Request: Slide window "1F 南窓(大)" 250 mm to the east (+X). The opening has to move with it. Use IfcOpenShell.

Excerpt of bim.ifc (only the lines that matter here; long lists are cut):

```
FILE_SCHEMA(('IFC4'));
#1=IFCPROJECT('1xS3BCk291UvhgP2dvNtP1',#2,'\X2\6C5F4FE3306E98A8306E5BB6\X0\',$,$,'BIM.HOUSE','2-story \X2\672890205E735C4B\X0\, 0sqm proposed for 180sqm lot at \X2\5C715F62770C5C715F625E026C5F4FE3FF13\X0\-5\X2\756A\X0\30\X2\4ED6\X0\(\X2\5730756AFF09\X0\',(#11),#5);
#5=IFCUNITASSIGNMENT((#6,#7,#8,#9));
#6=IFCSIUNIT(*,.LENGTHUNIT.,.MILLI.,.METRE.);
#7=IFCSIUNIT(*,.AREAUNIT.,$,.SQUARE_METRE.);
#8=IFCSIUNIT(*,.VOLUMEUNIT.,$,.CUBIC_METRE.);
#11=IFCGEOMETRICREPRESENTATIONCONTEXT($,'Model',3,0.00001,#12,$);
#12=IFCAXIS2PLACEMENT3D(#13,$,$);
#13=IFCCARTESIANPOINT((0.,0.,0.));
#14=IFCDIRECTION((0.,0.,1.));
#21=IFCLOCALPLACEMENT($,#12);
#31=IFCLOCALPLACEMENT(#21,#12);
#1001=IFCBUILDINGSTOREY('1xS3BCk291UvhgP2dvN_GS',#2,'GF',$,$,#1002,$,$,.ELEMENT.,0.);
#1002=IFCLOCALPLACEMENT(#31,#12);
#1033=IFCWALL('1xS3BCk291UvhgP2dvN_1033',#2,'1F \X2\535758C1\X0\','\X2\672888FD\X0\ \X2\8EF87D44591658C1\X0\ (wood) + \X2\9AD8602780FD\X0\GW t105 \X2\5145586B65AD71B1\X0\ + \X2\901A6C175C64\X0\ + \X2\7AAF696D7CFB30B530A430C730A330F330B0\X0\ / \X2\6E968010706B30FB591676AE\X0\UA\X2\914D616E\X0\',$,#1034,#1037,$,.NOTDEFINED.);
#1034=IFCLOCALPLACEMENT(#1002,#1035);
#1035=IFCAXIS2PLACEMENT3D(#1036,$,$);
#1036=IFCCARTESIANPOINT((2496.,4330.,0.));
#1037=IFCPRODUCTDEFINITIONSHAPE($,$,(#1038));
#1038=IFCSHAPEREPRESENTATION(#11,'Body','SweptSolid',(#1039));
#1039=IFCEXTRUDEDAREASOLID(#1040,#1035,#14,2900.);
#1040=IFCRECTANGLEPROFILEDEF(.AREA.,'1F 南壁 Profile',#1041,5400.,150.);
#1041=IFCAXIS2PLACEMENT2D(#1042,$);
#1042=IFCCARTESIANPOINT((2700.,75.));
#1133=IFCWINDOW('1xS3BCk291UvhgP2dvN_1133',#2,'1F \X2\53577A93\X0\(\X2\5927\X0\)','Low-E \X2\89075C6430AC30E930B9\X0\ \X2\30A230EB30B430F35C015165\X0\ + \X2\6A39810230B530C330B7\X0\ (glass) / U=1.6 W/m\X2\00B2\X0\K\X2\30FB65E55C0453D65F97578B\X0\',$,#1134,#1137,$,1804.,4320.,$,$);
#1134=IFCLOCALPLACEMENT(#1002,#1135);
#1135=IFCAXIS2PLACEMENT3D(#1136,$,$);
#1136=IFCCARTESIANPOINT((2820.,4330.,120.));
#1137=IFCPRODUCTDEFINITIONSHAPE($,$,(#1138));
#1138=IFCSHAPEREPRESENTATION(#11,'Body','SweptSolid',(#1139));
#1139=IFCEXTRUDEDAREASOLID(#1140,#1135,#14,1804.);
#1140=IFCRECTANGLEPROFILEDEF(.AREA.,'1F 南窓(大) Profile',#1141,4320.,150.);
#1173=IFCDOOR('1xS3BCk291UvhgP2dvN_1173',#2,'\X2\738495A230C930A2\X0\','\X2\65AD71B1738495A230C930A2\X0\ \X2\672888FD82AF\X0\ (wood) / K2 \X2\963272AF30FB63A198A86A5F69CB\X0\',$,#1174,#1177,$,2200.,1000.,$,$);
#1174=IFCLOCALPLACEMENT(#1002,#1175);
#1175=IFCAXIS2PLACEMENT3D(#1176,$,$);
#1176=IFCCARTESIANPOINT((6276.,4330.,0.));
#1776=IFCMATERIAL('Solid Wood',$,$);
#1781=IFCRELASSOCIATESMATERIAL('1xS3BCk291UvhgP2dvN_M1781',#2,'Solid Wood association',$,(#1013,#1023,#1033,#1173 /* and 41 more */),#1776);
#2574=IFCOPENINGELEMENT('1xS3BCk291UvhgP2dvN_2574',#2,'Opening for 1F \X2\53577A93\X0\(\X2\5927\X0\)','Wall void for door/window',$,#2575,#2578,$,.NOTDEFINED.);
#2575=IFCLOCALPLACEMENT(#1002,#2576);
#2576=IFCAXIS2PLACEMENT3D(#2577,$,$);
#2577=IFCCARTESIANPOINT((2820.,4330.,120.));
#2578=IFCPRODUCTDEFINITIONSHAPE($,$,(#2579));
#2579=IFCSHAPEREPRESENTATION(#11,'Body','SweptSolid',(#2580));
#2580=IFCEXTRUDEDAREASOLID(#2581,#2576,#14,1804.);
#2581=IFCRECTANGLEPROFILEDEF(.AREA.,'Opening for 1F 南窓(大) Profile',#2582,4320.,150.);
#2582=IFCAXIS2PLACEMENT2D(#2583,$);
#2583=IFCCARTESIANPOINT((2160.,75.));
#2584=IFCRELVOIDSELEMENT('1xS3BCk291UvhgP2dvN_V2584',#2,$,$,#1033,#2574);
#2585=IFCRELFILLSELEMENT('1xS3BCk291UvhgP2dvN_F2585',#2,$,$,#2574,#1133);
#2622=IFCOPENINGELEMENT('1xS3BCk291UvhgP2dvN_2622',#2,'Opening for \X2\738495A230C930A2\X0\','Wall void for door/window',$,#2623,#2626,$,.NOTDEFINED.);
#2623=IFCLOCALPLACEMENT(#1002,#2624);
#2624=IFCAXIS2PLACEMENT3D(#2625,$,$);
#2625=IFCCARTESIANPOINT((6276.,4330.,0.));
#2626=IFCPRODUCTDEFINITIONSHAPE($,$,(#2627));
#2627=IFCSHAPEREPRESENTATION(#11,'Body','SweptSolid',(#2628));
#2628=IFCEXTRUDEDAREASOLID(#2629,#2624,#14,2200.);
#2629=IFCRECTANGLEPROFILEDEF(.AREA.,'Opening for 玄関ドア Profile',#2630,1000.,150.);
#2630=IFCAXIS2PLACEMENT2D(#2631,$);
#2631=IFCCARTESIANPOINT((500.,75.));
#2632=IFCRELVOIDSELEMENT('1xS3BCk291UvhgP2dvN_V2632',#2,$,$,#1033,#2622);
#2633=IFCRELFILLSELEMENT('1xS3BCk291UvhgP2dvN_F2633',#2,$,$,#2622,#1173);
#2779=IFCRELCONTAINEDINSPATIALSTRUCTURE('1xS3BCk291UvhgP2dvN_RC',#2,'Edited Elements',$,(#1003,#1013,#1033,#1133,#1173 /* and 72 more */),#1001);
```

```python
import ifcopenshell
import ifcopenshell.api.geometry
import ifcopenshell.util.placement

model = ifcopenshell.open("bim.ifc")

window = model.by_id(1133)
opening = window.FillsVoids[0].RelatingOpeningElement
wall = opening.VoidsElements[0].RelatingBuildingElement

wall_matrix = ifcopenshell.util.placement.get_local_placement(wall.ObjectPlacement)
shift = wall_matrix[:3, 0] * 250.0
before = ifcopenshell.util.placement.get_local_placement(window.ObjectPlacement)[:3, 3].copy()

# The window is not placed relative to its opening, so move both.
for product in (opening, window):
    matrix = ifcopenshell.util.placement.get_local_placement(product.ObjectPlacement)
    matrix[:3, 3] += shift
    ifcopenshell.api.geometry.edit_object_placement(model, product=product, matrix=matrix, is_si=False)

after = ifcopenshell.util.placement.get_local_placement(window.ObjectPlacement)[:3, 3]
print("window moved by", (after - before).round(3) + 0.0)

model.write("bim_edited.ifc")
```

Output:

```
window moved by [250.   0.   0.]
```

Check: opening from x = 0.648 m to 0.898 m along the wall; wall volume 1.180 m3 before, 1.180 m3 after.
